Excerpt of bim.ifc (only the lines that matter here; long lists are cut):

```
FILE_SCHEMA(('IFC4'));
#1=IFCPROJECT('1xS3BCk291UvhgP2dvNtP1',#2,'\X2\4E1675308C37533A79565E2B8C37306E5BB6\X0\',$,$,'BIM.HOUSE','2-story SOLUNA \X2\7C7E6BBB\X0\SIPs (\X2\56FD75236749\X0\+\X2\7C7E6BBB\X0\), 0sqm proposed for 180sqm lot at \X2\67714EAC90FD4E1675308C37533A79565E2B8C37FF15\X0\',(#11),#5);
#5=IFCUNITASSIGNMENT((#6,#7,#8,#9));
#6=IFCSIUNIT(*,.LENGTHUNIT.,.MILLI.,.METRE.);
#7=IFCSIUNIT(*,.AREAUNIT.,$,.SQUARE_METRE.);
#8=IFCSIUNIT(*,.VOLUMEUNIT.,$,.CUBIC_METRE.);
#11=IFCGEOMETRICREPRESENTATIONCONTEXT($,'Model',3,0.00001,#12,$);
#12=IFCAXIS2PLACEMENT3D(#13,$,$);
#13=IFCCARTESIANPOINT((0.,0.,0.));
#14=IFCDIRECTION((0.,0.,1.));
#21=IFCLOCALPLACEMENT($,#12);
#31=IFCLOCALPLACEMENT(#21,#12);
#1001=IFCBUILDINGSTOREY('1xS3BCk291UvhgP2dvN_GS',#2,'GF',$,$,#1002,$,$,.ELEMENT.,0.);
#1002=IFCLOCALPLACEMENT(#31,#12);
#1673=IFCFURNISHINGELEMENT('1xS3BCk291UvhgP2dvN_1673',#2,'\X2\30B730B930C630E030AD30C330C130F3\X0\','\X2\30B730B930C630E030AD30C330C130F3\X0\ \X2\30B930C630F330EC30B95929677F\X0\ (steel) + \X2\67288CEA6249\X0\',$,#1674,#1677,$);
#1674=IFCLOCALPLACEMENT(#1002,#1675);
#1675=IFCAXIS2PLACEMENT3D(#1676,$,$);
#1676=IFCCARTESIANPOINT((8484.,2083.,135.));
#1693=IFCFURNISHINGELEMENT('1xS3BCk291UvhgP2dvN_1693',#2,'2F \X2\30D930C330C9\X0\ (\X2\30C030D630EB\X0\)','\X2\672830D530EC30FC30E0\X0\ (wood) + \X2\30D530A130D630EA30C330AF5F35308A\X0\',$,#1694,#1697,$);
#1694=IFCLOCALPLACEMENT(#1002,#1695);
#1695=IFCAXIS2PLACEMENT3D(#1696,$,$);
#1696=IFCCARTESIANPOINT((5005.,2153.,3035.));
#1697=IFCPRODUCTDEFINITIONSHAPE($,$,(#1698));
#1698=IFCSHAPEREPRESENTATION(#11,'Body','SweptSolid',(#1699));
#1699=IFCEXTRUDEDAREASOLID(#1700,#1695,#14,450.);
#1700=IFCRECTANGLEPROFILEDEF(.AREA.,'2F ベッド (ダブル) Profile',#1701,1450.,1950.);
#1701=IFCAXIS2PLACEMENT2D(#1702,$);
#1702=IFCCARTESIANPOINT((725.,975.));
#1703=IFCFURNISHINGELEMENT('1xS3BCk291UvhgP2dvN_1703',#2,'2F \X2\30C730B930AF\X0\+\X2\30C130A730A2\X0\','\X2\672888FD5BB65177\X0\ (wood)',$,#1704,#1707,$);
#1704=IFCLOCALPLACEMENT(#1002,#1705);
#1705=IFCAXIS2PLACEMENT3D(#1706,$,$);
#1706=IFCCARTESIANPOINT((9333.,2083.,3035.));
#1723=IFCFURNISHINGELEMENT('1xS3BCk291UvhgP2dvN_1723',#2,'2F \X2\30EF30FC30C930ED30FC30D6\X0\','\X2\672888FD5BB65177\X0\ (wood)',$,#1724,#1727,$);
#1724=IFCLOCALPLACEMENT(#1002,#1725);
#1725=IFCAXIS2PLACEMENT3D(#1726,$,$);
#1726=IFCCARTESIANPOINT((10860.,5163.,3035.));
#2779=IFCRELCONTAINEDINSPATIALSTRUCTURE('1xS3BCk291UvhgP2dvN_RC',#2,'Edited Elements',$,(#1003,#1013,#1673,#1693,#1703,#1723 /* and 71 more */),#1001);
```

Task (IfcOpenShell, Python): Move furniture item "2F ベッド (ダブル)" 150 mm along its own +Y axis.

```python
import ifcopenshell
import ifcopenshell.api.geometry
import ifcopenshell.util.placement
import ifcopenshell.util.unit

model = ifcopenshell.open("bim.ifc")
unit_scale = ifcopenshell.util.unit.calculate_unit_scale(model)

item = model.by_guid("1xS3BCk291UvhgP2dvN_1693")
matrix = ifcopenshell.util.placement.get_local_placement(item.ObjectPlacement)
matrix[:3, 3] += matrix[:3, 1] * 0.15 / unit_scale
ifcopenshell.api.geometry.edit_object_placement(model, product=item, matrix=matrix, is_si=False)

print(ifcopenshell.util.placement.get_local_placement(item.ObjectPlacement).round(3) + 0.0)

model.write("bim_updated.ifc")
```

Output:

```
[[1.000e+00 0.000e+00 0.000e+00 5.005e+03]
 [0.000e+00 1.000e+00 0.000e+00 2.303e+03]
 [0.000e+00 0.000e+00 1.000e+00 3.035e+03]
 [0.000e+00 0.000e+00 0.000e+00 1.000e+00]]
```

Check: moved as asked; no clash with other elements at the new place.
